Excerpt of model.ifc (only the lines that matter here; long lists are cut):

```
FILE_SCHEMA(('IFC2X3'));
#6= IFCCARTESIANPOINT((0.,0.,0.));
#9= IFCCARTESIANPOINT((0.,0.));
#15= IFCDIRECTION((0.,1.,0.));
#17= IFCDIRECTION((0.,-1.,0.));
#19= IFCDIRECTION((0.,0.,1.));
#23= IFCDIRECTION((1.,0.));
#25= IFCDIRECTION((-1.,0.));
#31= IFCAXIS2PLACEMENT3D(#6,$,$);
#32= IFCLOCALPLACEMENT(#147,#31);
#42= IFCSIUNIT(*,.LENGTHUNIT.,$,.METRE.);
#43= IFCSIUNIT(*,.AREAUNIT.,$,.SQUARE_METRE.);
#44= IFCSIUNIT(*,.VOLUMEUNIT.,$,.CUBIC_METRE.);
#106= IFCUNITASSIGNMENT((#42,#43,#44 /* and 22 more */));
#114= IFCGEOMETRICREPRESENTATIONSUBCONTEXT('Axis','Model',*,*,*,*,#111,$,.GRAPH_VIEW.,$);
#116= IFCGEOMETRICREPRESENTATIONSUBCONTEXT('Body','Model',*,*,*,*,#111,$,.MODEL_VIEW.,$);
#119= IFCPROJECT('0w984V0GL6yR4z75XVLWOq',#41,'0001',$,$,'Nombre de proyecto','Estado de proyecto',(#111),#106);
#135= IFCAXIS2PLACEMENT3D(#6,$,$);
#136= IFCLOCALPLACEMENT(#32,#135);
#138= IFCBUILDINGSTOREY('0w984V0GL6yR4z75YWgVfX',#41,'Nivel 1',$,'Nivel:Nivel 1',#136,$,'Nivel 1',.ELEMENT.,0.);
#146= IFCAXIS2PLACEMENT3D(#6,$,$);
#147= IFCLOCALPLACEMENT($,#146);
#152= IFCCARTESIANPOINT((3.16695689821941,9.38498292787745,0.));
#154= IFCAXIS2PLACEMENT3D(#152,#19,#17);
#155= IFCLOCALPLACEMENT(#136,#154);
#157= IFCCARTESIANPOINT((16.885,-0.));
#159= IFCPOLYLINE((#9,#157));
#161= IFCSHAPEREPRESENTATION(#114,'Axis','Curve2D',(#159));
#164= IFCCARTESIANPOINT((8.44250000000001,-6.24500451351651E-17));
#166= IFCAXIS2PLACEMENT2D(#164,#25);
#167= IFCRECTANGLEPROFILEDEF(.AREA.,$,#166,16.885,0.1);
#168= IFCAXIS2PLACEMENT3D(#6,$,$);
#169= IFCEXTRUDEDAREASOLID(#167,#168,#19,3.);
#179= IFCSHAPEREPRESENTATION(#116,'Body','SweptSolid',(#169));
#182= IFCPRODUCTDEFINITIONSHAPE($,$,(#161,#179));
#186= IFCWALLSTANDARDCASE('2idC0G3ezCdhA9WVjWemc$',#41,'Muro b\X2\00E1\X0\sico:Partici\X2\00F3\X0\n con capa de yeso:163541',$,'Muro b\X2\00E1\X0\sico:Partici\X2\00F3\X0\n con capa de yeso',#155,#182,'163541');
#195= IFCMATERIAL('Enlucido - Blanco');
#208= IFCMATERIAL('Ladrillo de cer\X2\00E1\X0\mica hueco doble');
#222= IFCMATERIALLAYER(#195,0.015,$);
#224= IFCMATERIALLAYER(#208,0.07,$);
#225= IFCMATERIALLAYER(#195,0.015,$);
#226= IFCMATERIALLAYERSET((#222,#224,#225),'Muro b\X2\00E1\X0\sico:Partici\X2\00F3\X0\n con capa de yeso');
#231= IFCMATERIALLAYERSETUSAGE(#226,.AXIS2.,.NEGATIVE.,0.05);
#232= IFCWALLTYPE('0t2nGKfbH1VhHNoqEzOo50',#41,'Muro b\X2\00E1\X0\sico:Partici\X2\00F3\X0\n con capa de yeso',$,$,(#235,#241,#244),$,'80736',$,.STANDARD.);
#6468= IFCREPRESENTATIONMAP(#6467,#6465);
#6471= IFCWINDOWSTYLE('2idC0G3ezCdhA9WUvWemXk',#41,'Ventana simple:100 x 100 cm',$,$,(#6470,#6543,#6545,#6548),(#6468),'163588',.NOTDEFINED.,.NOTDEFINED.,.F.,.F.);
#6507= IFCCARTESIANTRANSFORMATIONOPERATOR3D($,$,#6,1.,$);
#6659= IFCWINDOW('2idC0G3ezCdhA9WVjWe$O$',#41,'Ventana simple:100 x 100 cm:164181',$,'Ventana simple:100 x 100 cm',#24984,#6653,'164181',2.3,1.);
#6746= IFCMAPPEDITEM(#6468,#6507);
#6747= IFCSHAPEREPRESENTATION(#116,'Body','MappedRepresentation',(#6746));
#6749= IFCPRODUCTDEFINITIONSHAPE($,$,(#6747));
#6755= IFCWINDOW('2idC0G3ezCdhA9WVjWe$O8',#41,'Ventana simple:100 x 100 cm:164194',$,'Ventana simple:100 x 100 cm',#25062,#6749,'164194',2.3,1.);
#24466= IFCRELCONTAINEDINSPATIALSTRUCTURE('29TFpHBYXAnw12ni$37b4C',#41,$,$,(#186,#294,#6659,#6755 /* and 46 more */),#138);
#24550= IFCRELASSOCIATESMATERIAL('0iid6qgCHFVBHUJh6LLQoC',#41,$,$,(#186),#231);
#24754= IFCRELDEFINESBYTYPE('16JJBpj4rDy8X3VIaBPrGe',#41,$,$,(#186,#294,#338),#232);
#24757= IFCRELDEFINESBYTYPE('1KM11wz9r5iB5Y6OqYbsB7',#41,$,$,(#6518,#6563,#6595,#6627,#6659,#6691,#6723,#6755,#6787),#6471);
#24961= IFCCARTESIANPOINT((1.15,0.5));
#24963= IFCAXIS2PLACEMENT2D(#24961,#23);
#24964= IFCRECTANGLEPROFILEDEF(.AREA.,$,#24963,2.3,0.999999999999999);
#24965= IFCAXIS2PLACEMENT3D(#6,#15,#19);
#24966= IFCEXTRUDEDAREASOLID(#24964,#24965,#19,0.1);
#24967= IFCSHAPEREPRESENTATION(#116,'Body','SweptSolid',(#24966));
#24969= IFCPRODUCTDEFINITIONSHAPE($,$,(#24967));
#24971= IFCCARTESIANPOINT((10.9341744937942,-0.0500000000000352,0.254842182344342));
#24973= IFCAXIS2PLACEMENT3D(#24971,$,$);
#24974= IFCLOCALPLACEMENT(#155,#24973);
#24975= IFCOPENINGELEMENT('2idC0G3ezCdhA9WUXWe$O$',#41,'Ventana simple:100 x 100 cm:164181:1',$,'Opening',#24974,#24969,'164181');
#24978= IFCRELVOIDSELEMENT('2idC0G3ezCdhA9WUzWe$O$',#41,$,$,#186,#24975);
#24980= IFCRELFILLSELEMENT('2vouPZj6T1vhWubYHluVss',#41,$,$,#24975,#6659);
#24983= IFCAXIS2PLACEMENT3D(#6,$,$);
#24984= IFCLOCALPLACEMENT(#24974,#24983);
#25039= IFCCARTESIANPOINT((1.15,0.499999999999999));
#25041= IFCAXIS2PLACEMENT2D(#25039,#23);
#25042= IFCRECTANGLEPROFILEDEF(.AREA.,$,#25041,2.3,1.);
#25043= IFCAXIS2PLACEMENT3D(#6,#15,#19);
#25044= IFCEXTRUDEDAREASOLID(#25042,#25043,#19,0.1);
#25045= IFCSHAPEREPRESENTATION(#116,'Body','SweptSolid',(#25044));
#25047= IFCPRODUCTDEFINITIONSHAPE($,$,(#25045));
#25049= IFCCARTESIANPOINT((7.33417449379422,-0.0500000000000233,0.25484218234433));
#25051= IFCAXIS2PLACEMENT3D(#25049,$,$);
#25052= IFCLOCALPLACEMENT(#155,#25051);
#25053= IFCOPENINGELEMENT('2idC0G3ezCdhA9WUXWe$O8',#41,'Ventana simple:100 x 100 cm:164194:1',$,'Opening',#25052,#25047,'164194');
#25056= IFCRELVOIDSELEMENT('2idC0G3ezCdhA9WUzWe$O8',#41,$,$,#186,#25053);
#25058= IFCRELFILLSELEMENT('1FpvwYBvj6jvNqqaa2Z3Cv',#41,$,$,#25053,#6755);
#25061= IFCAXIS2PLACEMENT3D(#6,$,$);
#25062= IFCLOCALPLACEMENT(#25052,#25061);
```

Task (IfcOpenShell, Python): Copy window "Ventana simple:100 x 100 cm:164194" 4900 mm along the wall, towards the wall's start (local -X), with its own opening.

```python
import ifcopenshell
import ifcopenshell.api.feature
import ifcopenshell.api.geometry
import ifcopenshell.api.root
import ifcopenshell.geom
import ifcopenshell.util.element
import ifcopenshell.util.placement
import ifcopenshell.util.shape
import ifcopenshell.util.unit

model = ifcopenshell.open("model.ifc")
unit_scale = ifcopenshell.util.unit.calculate_unit_scale(model)
settings = ifcopenshell.geom.settings()


def volume(element):
    """Net volume in cubic metres, openings subtracted."""
    shape = ifcopenshell.geom.create_shape(settings, element)
    return ifcopenshell.util.shape.get_volume(shape.geometry)


def reuse_history(source, copy):
    """copy_class also copies each property set's owner history, people and application; keep the originals."""
    for rel in copy.IsDefinedBy:
        if rel.is_a("IfcRelDefinesByProperties") and (history := rel.RelatingPropertyDefinition.OwnerHistory):
            rel.RelatingPropertyDefinition.OwnerHistory = source.OwnerHistory
            ifcopenshell.util.element.remove_deep2(model, history)


window = model.by_guid("2idC0G3ezCdhA9WVjWe$O8")
opening = window.FillsVoids[0].RelatingOpeningElement
wall = opening.VoidsElements[0].RelatingBuildingElement
before = volume(wall)
shift = ifcopenshell.util.placement.get_local_placement(wall.ObjectPlacement)[:3, 0] * -4.9 / unit_scale

# copy_class copies the void relationship, type, container and properties, but no geometry.
new_opening = ifcopenshell.api.root.copy_class(model, product=opening)
new_opening.Representation = ifcopenshell.util.element.copy_deep(
    model, opening.Representation, exclude=["IfcGeometricRepresentationContext", "IfcRepresentationMap"]
)
new_opening.Name = "Ventana simple:100 x 100 cm"
new_opening.Tag = None
new_window = ifcopenshell.api.root.copy_class(model, product=window)
new_window.Representation = ifcopenshell.util.element.copy_deep(
    model, window.Representation, exclude=["IfcGeometricRepresentationContext", "IfcRepresentationMap"]
)
new_window.Name = "Ventana simple:100 x 100 cm"
new_window.Tag = None
reuse_history(window, new_window)
fills = ifcopenshell.api.feature.add_filling(model, opening=new_opening, element=new_window)
fills.OwnerHistory = new_window.OwnerHistory  # required in IFC2X3

for old, new in ((opening, new_opening), (window, new_window)):
    matrix = ifcopenshell.util.placement.get_local_placement(old.ObjectPlacement)
    matrix[:3, 3] += shift
    ifcopenshell.api.geometry.edit_object_placement(model, product=new, matrix=matrix, is_si=False)

after = volume(wall)

print(f"wall volume {before:.3f} -> {after:.3f} m3")

model.write("model-out.ifc")
```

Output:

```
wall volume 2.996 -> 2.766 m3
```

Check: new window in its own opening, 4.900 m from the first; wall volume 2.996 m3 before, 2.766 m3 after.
